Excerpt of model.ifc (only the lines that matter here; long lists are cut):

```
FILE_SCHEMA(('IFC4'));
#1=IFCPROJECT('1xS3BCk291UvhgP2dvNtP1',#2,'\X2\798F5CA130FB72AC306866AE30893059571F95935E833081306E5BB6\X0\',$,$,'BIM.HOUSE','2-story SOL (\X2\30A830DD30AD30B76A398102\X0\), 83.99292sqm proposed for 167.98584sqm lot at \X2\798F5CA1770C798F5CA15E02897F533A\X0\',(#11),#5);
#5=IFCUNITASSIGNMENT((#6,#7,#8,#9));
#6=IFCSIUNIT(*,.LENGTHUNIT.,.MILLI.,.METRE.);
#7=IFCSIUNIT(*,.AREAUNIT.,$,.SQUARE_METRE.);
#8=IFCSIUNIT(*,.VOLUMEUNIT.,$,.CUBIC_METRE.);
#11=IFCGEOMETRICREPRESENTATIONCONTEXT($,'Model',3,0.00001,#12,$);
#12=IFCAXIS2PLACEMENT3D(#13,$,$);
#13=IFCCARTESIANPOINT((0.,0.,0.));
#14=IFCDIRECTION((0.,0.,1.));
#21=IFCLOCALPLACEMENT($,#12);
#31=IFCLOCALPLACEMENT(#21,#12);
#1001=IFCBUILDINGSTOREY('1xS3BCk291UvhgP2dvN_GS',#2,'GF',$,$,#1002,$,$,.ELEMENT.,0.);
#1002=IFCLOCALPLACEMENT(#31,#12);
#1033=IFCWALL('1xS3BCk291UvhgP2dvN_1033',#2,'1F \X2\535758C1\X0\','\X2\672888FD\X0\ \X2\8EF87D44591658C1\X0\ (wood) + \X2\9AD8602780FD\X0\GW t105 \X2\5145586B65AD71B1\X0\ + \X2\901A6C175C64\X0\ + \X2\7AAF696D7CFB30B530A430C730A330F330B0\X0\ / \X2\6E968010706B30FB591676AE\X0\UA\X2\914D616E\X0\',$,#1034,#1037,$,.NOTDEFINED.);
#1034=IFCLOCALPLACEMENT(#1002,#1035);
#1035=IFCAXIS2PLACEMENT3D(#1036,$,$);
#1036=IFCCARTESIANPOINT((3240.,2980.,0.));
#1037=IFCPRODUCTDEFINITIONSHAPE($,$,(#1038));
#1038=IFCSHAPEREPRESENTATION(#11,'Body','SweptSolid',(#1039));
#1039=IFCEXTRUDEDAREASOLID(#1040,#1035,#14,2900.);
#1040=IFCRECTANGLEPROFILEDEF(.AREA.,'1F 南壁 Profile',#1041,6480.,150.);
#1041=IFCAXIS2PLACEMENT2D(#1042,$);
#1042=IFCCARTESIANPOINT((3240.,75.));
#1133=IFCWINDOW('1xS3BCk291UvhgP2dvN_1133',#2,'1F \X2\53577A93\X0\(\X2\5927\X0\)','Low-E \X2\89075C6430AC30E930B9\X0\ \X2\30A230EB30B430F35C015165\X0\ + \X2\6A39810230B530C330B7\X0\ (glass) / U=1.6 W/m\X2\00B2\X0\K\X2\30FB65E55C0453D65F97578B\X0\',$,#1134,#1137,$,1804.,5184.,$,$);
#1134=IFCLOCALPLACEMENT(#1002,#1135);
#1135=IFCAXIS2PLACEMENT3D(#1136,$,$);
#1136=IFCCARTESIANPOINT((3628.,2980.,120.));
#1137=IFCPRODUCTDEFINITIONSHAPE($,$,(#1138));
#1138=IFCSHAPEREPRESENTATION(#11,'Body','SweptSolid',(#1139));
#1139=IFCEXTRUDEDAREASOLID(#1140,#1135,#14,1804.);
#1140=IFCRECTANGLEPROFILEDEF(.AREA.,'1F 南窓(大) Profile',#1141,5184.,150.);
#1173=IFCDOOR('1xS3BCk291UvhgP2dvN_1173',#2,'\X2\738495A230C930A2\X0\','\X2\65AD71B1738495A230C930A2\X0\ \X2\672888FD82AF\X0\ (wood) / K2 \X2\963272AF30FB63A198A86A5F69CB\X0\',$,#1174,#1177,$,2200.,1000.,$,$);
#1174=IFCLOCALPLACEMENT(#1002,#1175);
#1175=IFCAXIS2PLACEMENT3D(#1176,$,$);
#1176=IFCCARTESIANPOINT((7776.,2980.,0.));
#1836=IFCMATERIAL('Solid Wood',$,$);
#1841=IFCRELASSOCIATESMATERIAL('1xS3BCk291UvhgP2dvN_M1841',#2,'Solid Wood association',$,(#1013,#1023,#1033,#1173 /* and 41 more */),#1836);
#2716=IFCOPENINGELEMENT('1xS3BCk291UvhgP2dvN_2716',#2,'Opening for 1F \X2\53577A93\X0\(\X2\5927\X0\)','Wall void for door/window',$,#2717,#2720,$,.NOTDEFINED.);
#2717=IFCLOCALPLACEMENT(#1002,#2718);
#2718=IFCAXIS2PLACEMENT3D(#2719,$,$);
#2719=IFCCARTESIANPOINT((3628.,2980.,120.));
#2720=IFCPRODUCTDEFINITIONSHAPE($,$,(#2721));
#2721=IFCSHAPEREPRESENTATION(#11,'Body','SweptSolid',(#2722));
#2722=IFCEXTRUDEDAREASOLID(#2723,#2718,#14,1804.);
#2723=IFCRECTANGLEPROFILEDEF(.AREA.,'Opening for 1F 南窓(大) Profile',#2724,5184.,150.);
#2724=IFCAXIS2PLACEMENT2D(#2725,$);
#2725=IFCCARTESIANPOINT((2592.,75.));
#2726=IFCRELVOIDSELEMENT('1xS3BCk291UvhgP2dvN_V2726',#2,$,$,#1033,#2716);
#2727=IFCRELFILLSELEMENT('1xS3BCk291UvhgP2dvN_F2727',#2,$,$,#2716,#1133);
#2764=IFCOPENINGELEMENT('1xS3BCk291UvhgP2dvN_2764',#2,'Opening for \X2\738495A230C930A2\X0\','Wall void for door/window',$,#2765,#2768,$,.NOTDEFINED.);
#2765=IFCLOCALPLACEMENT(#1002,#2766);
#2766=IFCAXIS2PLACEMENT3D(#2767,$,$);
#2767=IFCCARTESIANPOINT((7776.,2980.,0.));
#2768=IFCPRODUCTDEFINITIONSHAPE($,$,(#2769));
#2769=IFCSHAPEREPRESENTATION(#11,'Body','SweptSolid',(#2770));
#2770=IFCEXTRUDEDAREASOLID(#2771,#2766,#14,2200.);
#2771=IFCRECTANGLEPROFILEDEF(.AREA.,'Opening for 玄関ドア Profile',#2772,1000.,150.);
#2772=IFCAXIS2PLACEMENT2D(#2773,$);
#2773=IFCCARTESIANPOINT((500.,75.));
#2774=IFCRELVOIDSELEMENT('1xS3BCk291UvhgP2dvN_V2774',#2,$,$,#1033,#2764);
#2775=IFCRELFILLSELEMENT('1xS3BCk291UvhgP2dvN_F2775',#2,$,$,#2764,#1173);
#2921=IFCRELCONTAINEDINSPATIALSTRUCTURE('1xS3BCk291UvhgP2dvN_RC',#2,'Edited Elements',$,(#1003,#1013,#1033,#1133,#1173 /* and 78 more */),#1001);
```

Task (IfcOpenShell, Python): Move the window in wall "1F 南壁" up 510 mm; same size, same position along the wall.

```python
import numpy as np
import ifcopenshell
import ifcopenshell.api.geometry
import ifcopenshell.util.placement
import ifcopenshell.util.unit

model = ifcopenshell.open("model.ifc")
unit_scale = ifcopenshell.util.unit.calculate_unit_scale(model)

window = model.by_guid("1xS3BCk291UvhgP2dvN_1133")
opening = window.FillsVoids[0].RelatingOpeningElement
dz = 0.51 / unit_scale

shift = np.array([0.0, 0.0, dz])
# The window is not placed relative to its opening, so move both.
for product in (opening, window):
    matrix = ifcopenshell.util.placement.get_local_placement(product.ObjectPlacement)
    matrix[:3, 3] += shift
    ifcopenshell.api.geometry.edit_object_placement(model, product=product, matrix=matrix, is_si=False)

print(f"moved by {dz * unit_scale:+.3f} m")

model.write("model_updated.ifc")
```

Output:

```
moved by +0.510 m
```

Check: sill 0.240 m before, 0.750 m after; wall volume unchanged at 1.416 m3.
